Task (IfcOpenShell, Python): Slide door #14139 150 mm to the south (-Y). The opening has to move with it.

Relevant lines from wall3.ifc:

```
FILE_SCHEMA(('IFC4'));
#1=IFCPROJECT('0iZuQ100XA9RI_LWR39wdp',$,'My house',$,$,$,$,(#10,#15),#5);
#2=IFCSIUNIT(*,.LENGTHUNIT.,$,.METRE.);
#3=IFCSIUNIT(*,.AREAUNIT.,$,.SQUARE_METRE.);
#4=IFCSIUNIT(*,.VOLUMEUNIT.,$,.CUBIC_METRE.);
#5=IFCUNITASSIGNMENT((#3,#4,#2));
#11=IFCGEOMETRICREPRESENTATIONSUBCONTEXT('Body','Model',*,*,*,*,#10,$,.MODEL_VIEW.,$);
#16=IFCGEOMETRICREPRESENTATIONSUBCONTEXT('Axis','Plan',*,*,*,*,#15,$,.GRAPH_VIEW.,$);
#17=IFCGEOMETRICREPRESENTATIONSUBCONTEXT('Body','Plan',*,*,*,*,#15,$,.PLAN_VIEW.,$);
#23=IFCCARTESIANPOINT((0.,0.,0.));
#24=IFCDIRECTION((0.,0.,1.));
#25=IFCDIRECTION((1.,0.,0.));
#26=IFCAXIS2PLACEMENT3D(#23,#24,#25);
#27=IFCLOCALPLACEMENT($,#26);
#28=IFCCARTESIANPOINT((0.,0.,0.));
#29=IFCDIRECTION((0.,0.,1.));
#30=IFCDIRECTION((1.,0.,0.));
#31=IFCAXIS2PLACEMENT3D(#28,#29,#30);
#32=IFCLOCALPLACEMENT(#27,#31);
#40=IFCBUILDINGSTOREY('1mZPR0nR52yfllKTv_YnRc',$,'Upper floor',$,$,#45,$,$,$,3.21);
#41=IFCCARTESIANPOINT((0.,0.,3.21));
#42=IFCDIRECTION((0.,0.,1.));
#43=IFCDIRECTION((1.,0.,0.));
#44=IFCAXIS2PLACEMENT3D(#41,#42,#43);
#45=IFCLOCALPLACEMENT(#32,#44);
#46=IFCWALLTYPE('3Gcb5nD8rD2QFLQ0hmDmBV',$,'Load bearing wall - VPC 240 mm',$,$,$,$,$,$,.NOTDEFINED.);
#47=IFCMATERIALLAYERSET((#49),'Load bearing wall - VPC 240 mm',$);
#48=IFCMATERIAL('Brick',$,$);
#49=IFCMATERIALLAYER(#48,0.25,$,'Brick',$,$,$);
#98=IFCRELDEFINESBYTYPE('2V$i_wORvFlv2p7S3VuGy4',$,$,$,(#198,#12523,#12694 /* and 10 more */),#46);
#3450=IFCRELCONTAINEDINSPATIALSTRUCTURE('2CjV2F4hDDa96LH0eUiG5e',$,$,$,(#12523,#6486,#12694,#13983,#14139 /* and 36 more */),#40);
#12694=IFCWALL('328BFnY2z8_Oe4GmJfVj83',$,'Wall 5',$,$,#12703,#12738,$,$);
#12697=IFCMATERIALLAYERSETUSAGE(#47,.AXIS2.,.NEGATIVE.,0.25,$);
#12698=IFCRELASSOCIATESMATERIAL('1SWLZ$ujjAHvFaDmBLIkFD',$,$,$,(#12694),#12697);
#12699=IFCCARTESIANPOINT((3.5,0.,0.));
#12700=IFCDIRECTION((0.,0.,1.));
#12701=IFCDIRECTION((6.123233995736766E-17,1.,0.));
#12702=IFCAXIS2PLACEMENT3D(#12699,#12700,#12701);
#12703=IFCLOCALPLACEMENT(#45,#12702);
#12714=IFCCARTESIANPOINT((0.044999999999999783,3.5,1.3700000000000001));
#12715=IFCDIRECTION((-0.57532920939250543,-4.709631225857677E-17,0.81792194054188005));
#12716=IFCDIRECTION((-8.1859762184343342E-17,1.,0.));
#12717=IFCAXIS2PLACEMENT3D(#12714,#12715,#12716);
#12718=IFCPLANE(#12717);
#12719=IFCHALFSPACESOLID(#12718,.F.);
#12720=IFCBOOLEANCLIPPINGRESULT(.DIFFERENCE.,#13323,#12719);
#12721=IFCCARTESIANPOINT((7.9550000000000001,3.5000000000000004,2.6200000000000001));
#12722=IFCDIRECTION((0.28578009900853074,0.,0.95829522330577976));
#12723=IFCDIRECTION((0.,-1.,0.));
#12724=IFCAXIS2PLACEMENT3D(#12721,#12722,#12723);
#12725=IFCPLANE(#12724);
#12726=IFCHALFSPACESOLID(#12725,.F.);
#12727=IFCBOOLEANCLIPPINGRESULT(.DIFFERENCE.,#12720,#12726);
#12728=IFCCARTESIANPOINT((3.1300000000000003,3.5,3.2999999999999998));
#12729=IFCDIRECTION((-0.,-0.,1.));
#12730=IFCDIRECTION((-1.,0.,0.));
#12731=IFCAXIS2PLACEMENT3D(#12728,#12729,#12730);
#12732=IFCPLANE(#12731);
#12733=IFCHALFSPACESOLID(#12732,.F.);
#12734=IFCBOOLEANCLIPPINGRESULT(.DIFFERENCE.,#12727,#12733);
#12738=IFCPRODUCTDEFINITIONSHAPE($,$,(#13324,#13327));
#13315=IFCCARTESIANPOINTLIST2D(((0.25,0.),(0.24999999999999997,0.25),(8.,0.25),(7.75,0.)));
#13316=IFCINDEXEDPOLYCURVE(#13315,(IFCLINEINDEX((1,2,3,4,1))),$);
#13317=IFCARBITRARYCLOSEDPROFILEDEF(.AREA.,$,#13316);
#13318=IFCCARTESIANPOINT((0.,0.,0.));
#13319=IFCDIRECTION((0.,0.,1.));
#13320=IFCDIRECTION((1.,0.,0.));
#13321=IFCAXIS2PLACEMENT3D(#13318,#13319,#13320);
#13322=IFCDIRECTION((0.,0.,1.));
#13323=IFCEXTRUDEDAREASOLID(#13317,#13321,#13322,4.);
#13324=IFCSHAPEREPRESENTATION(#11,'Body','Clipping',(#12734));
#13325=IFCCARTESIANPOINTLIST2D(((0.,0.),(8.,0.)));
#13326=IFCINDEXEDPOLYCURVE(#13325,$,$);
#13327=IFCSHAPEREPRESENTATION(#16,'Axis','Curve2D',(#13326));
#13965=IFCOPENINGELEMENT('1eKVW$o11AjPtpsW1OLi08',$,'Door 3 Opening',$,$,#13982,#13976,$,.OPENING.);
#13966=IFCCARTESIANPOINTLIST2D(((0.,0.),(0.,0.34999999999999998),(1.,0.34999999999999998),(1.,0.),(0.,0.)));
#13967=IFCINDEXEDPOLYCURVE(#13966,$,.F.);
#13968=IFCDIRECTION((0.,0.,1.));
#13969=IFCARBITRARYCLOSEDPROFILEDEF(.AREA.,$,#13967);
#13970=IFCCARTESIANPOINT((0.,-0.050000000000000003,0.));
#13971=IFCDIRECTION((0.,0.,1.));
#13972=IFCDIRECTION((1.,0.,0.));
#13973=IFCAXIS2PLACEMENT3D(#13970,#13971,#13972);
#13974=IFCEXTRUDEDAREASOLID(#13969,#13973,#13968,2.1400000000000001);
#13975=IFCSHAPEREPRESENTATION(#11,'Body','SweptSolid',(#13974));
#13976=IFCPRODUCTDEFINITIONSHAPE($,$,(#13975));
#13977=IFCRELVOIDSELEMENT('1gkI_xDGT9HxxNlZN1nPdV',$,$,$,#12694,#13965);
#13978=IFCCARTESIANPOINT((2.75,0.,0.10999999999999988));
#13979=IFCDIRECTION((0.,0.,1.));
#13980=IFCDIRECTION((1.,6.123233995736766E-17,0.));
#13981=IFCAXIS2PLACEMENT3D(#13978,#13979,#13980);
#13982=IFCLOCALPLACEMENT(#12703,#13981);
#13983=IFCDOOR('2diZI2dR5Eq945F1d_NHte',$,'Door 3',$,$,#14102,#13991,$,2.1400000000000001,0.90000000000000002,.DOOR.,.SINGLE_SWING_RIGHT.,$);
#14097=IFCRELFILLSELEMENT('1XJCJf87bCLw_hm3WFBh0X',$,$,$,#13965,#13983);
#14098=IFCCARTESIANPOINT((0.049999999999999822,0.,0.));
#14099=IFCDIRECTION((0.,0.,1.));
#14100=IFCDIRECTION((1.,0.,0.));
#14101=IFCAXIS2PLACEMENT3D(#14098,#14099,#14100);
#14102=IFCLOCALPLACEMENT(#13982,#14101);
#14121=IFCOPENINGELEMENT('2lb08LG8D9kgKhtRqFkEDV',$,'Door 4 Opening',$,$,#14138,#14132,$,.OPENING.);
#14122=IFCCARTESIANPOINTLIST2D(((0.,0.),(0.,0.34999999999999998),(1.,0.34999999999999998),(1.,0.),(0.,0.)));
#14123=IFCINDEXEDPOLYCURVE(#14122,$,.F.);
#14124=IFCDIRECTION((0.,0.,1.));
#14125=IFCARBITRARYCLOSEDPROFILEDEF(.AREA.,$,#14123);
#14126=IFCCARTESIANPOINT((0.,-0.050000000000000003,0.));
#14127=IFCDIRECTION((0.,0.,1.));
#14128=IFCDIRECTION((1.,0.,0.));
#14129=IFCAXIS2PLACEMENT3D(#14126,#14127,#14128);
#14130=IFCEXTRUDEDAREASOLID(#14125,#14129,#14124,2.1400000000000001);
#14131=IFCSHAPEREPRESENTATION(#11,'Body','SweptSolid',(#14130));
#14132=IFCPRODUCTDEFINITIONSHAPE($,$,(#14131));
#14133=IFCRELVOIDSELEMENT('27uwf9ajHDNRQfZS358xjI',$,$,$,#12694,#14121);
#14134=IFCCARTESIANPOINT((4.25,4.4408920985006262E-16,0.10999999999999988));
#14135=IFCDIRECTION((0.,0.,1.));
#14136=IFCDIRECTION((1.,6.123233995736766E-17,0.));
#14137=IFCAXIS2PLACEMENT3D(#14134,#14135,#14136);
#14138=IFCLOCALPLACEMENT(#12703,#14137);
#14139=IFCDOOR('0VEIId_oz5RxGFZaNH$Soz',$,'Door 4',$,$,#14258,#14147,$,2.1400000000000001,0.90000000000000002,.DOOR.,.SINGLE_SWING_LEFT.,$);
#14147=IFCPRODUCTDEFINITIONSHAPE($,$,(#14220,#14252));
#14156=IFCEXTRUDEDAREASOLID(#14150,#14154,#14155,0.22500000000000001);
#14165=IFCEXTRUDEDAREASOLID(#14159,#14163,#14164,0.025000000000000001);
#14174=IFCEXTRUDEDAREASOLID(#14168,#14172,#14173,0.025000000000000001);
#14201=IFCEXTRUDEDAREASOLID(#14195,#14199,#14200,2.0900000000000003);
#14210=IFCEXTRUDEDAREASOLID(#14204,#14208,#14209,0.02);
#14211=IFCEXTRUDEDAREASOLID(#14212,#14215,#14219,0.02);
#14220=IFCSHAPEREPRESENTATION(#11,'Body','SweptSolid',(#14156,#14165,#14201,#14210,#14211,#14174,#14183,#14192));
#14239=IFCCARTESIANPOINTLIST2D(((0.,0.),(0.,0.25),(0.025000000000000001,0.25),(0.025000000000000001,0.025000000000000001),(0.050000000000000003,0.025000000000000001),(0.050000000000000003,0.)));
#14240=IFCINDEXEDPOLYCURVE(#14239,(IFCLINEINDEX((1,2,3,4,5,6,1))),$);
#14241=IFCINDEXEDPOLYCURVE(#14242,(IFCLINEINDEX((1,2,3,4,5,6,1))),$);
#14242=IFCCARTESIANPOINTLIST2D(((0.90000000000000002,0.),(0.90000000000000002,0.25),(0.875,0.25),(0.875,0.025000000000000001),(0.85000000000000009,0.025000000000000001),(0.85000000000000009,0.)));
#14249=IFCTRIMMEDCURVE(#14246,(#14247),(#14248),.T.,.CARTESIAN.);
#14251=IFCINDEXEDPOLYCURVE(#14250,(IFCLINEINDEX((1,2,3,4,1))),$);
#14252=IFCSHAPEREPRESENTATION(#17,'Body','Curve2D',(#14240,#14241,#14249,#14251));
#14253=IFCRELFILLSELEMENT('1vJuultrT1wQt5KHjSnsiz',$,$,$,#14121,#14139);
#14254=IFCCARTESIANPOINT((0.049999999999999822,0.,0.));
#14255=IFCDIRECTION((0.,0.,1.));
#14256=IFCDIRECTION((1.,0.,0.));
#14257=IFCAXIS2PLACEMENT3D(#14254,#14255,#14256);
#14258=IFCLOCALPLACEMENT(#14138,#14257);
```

```python
import ifcopenshell
import ifcopenshell.api.geometry
import ifcopenshell.util.placement

model = ifcopenshell.open("wall3.ifc")

door = model.by_guid("0VEIId_oz5RxGFZaNH$Soz")
opening = door.FillsVoids[0].RelatingOpeningElement
wall = opening.VoidsElements[0].RelatingBuildingElement

wall_matrix = ifcopenshell.util.placement.get_local_placement(wall.ObjectPlacement)
shift = wall_matrix[:3, 0] * -0.15
before = ifcopenshell.util.placement.get_local_placement(door.ObjectPlacement)[:3, 3].copy()

# The door is placed relative to its opening, so it follows when the opening moves.
matrix = ifcopenshell.util.placement.get_local_placement(opening.ObjectPlacement)
matrix[:3, 3] += shift
ifcopenshell.api.geometry.edit_object_placement(
    model, product=opening, matrix=matrix, is_si=False, should_transform_children=True
)

after = ifcopenshell.util.placement.get_local_placement(door.ObjectPlacement)[:3, 3]
print("door moved by", (after - before).round(3) + 0.0)

model.write("wall3_v2.ifc")
```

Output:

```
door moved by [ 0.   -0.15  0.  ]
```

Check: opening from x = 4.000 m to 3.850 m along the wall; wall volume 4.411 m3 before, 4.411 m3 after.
